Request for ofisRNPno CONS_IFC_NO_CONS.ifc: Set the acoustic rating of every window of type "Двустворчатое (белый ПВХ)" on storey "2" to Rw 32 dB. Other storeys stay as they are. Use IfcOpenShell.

First a look at what the model holds.

```python
import ifcopenshell
import ifcopenshell.util.element

model = ifcopenshell.open("ofisRNPno CONS_IFC_NO_CONS.ifc")
print(model.schema)
storey = next(s for s in model.by_type("IfcBuildingStorey") if s.Name == "2")
windows = [e for e in ifcopenshell.util.element.get_decomposition(storey) if e.is_a("IfcWindow")]
seen = {}
for e in windows:
    element_type = ifcopenshell.util.element.get_type(e)
    key = (element_type.Name if element_type != e and element_type else None, ifcopenshell.util.element.get_pset(e, "Pset_WindowCommon", "AcousticRating"))
    seen[key] = seen.get(key, 0) + 1
for (name, value), count in sorted(seen.items(), key=str):
    print(count, "x", name, "|", value)
```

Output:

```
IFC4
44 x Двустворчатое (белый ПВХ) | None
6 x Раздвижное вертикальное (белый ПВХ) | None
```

```python
import ifcopenshell
import ifcopenshell.api.pset
import ifcopenshell.util.element

model = ifcopenshell.open("ofisRNPno CONS_IFC_NO_CONS.ifc")

storey = next(s for s in model.by_type("IfcBuildingStorey") if s.Name == "2")
windows = [e for e in ifcopenshell.util.element.get_decomposition(storey) if e.is_a("IfcWindow")]

count = 0
for e in windows:
    element_type = ifcopenshell.util.element.get_type(e)
    if element_type in (None, e) or element_type.Name != "Двустворчатое (белый ПВХ)":
        continue
    # add_pset returns the element's existing set when there is one.
    pset = ifcopenshell.api.pset.add_pset(model, product=e, name="Pset_WindowCommon")
    ifcopenshell.api.pset.edit_pset(model, pset=pset, properties={"AcousticRating": "Rw 32 dB"})
    count += 1

print(count, "windows updated")

model.write("ofisRNPno CONS_IFC_NO_CONS_rev.ifc")
```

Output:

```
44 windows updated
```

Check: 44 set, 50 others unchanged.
